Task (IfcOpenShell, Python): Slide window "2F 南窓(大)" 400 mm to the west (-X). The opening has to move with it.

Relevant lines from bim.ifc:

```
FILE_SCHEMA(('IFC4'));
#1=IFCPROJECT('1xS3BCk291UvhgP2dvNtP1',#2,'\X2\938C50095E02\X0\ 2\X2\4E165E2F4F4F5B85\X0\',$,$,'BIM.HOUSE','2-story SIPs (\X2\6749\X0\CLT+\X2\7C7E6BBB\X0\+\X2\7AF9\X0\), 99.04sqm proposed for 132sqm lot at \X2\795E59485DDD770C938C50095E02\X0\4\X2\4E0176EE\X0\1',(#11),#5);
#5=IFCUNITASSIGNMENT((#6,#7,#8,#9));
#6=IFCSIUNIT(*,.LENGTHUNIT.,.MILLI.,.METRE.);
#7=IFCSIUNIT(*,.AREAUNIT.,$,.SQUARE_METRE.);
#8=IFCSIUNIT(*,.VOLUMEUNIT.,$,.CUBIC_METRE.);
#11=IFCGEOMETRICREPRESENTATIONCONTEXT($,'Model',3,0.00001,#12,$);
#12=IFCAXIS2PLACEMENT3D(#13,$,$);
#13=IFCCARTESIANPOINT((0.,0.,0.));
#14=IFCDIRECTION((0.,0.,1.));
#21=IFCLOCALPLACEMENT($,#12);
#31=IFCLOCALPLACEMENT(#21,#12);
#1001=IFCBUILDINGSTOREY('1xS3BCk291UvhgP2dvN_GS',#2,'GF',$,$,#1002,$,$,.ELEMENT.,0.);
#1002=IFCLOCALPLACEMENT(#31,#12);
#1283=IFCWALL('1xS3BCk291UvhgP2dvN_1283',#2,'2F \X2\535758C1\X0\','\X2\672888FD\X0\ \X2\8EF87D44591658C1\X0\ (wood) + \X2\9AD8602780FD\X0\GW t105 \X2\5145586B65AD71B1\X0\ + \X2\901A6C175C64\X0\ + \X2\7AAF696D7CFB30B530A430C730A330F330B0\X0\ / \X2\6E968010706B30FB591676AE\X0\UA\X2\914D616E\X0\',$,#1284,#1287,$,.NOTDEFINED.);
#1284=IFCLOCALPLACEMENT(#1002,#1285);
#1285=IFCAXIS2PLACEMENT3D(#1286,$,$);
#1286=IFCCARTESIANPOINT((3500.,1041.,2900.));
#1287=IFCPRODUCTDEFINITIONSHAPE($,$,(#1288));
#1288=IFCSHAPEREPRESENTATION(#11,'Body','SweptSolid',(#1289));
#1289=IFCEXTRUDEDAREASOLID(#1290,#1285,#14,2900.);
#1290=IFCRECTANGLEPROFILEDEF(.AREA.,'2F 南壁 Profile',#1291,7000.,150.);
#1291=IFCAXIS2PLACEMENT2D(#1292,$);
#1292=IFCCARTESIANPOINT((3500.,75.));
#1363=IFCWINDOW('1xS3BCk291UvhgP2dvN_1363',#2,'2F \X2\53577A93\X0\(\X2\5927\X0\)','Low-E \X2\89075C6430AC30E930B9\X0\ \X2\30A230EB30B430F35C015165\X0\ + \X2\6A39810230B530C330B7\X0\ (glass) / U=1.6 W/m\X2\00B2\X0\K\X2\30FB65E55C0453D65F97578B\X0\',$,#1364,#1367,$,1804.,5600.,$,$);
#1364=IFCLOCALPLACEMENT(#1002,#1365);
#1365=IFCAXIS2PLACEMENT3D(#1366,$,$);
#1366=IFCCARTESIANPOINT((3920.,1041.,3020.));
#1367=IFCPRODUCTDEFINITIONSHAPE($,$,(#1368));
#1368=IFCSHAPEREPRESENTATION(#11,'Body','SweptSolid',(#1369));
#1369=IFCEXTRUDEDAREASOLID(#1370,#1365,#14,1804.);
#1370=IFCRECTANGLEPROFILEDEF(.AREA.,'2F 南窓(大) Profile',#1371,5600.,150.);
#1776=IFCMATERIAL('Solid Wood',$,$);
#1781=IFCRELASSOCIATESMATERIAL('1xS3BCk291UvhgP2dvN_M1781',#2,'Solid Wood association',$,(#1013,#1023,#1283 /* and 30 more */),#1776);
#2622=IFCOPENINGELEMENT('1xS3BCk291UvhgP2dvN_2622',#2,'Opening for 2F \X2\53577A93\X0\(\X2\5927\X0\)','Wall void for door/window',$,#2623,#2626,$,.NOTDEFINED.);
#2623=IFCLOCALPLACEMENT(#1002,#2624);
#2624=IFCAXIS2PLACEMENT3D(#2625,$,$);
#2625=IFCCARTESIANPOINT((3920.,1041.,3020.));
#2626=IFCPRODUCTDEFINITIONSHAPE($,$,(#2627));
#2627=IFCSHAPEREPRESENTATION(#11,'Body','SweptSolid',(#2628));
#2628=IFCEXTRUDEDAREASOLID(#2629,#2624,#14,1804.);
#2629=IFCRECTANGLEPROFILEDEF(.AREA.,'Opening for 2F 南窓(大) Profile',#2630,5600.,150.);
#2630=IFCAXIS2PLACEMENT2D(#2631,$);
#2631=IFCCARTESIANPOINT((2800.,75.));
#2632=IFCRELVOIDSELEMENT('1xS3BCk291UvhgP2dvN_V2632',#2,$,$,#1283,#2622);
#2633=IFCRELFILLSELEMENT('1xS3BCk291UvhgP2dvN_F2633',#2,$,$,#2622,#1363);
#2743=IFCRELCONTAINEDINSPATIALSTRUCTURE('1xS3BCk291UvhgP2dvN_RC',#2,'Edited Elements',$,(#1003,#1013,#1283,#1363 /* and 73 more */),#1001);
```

```python
import ifcopenshell
import ifcopenshell.api.geometry
import ifcopenshell.util.placement
import ifcopenshell.util.unit

model = ifcopenshell.open("bim.ifc")
unit_scale = ifcopenshell.util.unit.calculate_unit_scale(model)

window = model.by_id(1363)
opening = window.FillsVoids[0].RelatingOpeningElement
wall = opening.VoidsElements[0].RelatingBuildingElement

wall_matrix = ifcopenshell.util.placement.get_local_placement(wall.ObjectPlacement)
shift = wall_matrix[:3, 0] * -0.4 / unit_scale
before = ifcopenshell.util.placement.get_local_placement(window.ObjectPlacement)[:3, 3].copy()

# The window is not placed relative to its opening, so move both.
for product in (opening, window):
    matrix = ifcopenshell.util.placement.get_local_placement(product.ObjectPlacement)
    matrix[:3, 3] += shift
    ifcopenshell.api.geometry.edit_object_placement(model, product=product, matrix=matrix, is_si=False)

after = ifcopenshell.util.placement.get_local_placement(window.ObjectPlacement)[:3, 3]
print("window moved by", (after - before).round(3) + 0.0)

model.write("bim-out.ifc")
```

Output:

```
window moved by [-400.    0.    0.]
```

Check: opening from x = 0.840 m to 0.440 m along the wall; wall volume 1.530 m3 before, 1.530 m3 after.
